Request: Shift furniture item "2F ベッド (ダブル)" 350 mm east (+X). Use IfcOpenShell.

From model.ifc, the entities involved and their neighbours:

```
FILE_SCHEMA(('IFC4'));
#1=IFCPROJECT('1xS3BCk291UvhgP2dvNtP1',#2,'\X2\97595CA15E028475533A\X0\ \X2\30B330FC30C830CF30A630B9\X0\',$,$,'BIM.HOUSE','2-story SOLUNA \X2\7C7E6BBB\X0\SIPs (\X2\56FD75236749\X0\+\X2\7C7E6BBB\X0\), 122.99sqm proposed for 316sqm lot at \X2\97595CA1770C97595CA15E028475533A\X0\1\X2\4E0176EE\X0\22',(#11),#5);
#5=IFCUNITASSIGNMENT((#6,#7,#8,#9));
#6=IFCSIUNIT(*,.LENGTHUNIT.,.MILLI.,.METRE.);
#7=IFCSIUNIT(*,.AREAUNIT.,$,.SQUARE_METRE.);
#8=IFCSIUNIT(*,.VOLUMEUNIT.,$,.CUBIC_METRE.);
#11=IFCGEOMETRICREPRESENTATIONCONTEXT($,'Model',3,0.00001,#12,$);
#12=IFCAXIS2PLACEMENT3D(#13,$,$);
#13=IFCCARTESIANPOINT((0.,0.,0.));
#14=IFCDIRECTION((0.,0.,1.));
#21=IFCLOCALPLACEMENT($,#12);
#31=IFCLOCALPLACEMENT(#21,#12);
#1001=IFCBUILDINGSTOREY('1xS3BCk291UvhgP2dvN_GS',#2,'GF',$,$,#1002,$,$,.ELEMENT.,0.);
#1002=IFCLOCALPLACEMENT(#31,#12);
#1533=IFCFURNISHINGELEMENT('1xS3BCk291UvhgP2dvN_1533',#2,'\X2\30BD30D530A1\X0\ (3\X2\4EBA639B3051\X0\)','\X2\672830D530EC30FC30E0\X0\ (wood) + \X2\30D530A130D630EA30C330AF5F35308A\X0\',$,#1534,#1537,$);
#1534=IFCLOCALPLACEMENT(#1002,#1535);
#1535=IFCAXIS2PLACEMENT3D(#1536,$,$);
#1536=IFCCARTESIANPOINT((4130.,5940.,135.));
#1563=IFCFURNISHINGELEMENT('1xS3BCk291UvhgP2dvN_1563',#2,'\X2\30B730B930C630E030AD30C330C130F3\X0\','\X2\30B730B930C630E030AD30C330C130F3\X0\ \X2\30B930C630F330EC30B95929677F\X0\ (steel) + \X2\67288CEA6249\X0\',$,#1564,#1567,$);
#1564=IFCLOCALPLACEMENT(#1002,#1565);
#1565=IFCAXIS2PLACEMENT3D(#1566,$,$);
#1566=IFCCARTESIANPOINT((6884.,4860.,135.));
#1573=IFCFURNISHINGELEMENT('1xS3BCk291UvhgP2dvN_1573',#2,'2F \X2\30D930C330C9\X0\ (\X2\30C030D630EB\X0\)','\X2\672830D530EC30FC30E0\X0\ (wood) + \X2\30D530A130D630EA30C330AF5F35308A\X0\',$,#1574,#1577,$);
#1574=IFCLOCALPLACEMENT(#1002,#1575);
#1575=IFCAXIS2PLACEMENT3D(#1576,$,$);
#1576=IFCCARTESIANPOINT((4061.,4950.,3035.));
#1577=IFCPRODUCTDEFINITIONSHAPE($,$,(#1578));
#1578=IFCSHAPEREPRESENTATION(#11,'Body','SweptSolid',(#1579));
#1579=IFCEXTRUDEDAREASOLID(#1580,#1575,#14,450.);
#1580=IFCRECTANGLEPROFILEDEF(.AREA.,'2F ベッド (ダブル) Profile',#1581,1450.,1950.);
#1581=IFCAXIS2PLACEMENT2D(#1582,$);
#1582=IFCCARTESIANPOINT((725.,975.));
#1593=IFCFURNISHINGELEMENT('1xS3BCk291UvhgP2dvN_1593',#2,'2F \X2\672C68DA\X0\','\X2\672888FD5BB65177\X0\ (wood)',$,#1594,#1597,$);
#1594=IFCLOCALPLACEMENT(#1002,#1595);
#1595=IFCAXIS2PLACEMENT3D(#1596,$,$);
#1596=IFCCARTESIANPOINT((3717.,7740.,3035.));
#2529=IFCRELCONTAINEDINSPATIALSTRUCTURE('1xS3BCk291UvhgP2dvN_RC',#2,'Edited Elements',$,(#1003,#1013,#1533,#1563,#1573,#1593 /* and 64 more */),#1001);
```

```python
import ifcopenshell
import ifcopenshell.api.geometry
import ifcopenshell.util.placement

model = ifcopenshell.open("model.ifc")

item = model.by_id(1573)
matrix = ifcopenshell.util.placement.get_local_placement(item.ObjectPlacement)
matrix[0, 3] += 350.0
ifcopenshell.api.geometry.edit_object_placement(model, product=item, matrix=matrix, is_si=False)

print(ifcopenshell.util.placement.get_local_placement(item.ObjectPlacement).round(3) + 0.0)

model.write("model_edited.ifc")
```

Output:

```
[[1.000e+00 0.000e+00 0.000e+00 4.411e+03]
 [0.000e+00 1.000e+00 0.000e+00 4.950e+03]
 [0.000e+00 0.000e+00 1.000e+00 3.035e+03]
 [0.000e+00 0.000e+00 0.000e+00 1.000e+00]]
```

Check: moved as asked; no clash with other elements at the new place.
